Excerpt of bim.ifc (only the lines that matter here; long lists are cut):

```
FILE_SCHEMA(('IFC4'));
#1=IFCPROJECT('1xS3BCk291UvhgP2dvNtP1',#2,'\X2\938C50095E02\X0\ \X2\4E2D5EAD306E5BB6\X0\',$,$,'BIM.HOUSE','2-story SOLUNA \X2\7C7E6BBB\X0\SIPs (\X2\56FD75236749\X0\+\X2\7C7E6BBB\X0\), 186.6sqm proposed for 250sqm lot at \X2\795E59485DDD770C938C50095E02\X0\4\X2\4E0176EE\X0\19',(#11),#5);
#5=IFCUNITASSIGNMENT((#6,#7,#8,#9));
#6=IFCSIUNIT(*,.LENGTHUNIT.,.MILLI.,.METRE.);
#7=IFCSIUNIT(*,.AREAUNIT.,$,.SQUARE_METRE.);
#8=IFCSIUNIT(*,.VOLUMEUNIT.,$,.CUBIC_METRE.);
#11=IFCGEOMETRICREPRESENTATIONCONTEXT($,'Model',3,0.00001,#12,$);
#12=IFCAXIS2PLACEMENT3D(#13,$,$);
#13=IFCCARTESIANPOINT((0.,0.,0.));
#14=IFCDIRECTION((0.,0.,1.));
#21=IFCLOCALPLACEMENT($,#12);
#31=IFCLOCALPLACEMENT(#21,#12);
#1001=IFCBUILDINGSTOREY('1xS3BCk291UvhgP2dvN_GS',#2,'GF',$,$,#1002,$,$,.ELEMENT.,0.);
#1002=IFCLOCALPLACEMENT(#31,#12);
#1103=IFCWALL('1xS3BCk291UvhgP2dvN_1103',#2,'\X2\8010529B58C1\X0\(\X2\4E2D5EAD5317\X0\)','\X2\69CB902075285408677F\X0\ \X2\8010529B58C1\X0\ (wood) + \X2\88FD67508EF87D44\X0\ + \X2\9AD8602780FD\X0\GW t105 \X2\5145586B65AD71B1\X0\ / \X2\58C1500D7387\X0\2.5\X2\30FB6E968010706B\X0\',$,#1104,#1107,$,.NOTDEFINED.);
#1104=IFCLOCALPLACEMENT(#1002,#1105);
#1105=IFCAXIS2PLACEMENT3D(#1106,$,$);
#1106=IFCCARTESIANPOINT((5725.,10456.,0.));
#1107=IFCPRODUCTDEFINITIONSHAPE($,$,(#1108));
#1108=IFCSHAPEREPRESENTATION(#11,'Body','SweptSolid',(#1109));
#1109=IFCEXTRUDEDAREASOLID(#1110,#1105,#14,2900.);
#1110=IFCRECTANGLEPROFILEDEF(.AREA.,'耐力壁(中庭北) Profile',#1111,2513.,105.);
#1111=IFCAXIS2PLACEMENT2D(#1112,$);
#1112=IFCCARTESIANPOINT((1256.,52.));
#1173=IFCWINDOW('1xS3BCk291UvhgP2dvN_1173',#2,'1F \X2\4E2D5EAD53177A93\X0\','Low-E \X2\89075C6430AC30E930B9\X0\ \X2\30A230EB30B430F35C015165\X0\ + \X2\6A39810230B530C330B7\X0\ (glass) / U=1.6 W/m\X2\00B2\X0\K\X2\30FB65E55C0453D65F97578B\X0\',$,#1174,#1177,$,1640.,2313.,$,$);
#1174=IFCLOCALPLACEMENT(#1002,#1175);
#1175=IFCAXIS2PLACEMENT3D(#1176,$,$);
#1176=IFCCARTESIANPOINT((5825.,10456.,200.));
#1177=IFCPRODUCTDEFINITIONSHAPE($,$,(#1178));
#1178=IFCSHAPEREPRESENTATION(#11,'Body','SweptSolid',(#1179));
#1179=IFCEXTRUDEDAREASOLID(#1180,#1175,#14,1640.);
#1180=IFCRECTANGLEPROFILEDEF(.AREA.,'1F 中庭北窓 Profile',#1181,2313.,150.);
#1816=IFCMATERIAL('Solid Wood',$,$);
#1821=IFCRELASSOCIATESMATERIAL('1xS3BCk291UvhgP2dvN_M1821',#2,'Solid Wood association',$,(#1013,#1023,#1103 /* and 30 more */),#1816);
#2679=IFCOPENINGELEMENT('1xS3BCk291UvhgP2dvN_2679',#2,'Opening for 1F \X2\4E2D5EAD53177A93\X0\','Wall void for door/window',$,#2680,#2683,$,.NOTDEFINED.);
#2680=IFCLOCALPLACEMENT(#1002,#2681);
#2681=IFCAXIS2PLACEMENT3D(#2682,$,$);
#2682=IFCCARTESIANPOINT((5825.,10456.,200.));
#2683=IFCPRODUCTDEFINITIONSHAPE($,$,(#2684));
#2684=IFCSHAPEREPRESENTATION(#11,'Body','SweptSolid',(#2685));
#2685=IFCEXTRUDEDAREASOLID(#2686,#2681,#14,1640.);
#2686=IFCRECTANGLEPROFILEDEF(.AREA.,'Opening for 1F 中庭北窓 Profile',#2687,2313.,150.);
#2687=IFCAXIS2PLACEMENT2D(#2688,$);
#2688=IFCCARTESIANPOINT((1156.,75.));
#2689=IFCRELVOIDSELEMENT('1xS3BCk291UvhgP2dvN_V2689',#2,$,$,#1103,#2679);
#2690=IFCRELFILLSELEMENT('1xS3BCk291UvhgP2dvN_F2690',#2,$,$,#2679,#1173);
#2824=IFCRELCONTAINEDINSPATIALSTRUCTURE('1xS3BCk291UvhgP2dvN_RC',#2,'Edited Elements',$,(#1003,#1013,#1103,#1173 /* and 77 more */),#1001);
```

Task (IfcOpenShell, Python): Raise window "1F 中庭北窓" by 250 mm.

```python
import numpy as np
import ifcopenshell
import ifcopenshell.api.geometry
import ifcopenshell.util.placement
import ifcopenshell.util.unit

model = ifcopenshell.open("bim.ifc")
unit_scale = ifcopenshell.util.unit.calculate_unit_scale(model)

window = model.by_guid("1xS3BCk291UvhgP2dvN_1173")
opening = window.FillsVoids[0].RelatingOpeningElement
dz = 250.0

shift = np.array([0.0, 0.0, dz])
# The window is not placed relative to its opening, so move both.
for product in (opening, window):
    matrix = ifcopenshell.util.placement.get_local_placement(product.ObjectPlacement)
    matrix[:3, 3] += shift
    ifcopenshell.api.geometry.edit_object_placement(model, product=product, matrix=matrix, is_si=False)

print(f"moved by {dz * unit_scale:+.3f} m")

model.write("bim_updated.ifc")
```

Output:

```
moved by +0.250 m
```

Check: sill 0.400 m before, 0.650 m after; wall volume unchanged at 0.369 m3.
